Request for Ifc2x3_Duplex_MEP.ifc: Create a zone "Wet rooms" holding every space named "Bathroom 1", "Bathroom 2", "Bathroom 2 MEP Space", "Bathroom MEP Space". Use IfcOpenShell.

First a look at what the model holds.

```python
import ifcopenshell

model = ifcopenshell.open("Ifc2x3_Duplex_MEP.ifc")
print(model.schema)
seen = {}
for space in model.by_type("IfcSpace"):
    seen[space.LongName] = seen.get(space.LongName, 0) + 1
for name, count in sorted(seen.items(), key=str):
    print(count, "x", name)
print("zones:", [z.Name for z in model.by_type("IfcZone")][:20])
```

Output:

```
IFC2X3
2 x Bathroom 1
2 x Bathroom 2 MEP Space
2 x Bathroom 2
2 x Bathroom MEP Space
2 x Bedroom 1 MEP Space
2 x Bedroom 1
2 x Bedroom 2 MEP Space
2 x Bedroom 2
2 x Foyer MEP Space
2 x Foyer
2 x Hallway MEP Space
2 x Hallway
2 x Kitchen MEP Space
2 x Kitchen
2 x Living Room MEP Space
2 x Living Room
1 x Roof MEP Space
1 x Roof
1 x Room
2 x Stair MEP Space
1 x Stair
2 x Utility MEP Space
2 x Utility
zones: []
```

```python
import ifcopenshell
import ifcopenshell.api.group
import ifcopenshell.api.root

model = ifcopenshell.open("Ifc2x3_Duplex_MEP.ifc")

names = {"Bathroom 1", "Bathroom 2", "Bathroom 2 MEP Space", "Bathroom MEP Space"}
spaces = [s for s in model.by_type("IfcSpace") if s.LongName in names]

zone = ifcopenshell.api.root.create_entity(model, ifc_class="IfcZone", name="Wet rooms")
ifcopenshell.api.group.assign_group(model, products=spaces, group=zone)
print(len(spaces), "spaces in", zone.Name)

model.write("Ifc2x3_Duplex_MEP-out.ifc")
```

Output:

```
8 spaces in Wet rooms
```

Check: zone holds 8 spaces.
